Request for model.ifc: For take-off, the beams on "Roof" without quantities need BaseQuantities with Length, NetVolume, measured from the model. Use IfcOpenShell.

First a look at what the model holds.

```python
import ifcopenshell
import ifcopenshell.util.element
import ifcopenshell.util.unit

model = ifcopenshell.open("model.ifc")
print(model.schema)
for unit_type in ("LENGTHUNIT", "AREAUNIT", "VOLUMEUNIT"):
    print(unit_type, ifcopenshell.util.unit.calculate_unit_scale(model, unit_type))
storey = next(s for s in model.by_type("IfcBuildingStorey") if s.Name == "Roof")
beams = [e for e in ifcopenshell.util.element.get_decomposition(storey) if e.is_a("IfcBeam")]
for e in sorted(beams, key=lambda e: e.id()):
    print(e.id(), e.is_a(), e.Name, list(ifcopenshell.util.element.get_psets(e, qtos_only=True)), sep=" | ")
```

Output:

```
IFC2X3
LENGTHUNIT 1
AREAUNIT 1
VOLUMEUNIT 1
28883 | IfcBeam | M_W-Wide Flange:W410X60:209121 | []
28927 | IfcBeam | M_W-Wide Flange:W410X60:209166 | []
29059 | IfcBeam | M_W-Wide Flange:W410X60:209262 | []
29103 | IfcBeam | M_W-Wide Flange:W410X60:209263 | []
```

```python
import ifcopenshell
import ifcopenshell.api.pset
import ifcopenshell.geom
import ifcopenshell.util.element
import ifcopenshell.util.shape
import ifcopenshell.util.unit

model = ifcopenshell.open("model.ifc")
unit_scale = ifcopenshell.util.unit.calculate_unit_scale(model)
volume_scale = ifcopenshell.util.unit.calculate_unit_scale(model, "VOLUMEUNIT")
settings = ifcopenshell.geom.settings()

storey = next(s for s in model.by_type("IfcBuildingStorey") if s.Name == "Roof")
beams = [e for e in ifcopenshell.util.element.get_decomposition(storey) if e.is_a("IfcBeam")]

for e in sorted(beams, key=lambda e: e.id()):
    if ifcopenshell.util.element.get_psets(e, qtos_only=True, should_inherit=False):
        continue
    # Geometry comes back in metres, in the element's own axes.
    shape = ifcopenshell.geom.create_shape(settings, e)
    values = {
        "Length": ifcopenshell.util.shape.get_max_xyz(shape.geometry) / unit_scale,
        "NetVolume": ifcopenshell.util.shape.get_volume(shape.geometry) / volume_scale,
    }
    qto = ifcopenshell.api.pset.add_qto(model, product=e, name="BaseQuantities")
    ifcopenshell.api.pset.edit_qto(model, qto=qto, properties=values)
    print(e.id(), {k: round(v, 3) for k, v in values.items()})

model.write("model_rev.ifc")
```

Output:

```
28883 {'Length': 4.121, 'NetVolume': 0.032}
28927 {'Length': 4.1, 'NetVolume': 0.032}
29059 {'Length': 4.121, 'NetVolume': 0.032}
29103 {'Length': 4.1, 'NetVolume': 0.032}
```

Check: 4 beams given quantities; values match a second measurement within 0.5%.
